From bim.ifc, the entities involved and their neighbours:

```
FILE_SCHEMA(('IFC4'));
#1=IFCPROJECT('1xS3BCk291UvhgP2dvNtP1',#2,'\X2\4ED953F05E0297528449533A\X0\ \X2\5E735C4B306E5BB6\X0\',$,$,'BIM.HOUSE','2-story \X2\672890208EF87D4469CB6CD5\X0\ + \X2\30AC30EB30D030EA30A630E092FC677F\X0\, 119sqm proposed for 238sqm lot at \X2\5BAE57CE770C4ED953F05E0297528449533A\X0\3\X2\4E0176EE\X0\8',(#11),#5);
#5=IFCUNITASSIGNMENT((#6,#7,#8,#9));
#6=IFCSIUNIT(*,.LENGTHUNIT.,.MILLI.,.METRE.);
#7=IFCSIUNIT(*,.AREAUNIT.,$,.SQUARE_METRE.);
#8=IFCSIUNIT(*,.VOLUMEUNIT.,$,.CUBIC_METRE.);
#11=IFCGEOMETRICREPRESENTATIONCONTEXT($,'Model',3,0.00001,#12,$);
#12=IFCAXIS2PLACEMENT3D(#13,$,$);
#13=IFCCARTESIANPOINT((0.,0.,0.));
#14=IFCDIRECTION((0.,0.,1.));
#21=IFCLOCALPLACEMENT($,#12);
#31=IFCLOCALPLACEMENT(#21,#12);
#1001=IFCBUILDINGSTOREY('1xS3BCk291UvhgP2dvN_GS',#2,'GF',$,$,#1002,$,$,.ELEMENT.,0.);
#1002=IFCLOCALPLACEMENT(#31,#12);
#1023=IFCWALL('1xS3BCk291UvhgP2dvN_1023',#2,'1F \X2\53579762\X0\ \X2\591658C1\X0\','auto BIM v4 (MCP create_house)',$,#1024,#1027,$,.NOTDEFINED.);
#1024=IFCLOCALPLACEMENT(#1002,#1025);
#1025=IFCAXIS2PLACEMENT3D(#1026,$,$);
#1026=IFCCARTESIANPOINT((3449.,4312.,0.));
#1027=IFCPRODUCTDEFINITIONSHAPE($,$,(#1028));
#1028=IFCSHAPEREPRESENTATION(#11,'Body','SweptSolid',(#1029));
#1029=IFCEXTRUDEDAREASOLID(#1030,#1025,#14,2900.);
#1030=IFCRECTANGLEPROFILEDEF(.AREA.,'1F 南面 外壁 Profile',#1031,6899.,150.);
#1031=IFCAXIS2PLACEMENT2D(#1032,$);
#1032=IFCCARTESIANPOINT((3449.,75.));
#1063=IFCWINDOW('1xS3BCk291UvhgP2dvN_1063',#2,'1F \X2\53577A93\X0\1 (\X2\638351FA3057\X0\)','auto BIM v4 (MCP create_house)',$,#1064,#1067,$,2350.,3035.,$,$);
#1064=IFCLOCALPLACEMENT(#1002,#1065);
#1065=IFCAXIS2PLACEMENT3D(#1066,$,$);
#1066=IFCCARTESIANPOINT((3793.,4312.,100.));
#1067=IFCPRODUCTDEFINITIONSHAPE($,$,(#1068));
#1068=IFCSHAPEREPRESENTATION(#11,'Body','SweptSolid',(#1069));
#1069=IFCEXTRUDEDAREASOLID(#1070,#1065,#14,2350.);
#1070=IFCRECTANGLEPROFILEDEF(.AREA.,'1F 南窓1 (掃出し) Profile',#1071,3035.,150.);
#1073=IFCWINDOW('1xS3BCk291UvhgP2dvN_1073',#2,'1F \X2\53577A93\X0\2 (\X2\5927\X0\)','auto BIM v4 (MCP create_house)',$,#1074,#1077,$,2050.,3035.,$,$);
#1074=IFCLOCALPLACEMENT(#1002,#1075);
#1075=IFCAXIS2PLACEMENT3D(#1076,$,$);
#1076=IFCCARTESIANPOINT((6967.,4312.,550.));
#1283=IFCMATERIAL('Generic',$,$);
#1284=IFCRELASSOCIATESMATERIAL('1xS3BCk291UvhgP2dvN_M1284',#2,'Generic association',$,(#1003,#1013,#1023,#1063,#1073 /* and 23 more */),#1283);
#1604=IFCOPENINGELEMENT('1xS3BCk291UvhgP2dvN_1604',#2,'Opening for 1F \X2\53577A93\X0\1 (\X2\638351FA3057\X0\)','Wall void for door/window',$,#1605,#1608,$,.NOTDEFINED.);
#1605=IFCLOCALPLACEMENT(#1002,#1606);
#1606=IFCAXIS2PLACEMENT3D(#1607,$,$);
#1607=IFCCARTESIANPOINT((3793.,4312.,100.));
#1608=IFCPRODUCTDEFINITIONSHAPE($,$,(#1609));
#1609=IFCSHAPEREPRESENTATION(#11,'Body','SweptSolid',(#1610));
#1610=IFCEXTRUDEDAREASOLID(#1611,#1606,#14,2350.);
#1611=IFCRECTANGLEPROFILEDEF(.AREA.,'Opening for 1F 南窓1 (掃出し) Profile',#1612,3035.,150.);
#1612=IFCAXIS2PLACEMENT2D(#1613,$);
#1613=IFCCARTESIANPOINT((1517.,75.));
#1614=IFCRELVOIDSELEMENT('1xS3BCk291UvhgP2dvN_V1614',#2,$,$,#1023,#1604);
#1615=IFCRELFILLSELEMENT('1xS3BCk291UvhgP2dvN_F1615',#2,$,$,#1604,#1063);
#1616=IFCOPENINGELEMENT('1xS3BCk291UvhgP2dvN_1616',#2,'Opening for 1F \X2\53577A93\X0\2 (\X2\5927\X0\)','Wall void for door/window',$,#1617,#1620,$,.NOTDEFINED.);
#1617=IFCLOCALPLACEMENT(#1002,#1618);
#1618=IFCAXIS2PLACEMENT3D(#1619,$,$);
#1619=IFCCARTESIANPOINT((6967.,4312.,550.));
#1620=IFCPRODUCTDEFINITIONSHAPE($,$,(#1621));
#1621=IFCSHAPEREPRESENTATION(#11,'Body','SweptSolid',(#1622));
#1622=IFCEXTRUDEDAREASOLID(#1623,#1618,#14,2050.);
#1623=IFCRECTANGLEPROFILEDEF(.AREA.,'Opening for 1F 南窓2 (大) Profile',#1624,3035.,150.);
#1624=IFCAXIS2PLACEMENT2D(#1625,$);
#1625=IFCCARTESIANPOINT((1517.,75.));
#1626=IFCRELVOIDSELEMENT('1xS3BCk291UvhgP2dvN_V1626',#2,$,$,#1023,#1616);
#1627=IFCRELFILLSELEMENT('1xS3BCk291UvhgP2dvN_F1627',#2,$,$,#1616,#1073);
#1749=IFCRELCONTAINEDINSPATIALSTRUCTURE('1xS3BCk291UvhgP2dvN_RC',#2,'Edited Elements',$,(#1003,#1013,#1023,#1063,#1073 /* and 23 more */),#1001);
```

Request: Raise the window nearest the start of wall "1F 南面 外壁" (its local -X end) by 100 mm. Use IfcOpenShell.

```python
import numpy as np
import ifcopenshell
import ifcopenshell.api.geometry
import ifcopenshell.util.placement
import ifcopenshell.util.unit

model = ifcopenshell.open("bim.ifc")
unit_scale = ifcopenshell.util.unit.calculate_unit_scale(model)

window = model.by_guid("1xS3BCk291UvhgP2dvN_1063")
opening = window.FillsVoids[0].RelatingOpeningElement
dz = 0.1 / unit_scale

shift = np.array([0.0, 0.0, dz])
# The window is not placed relative to its opening, so move both.
for product in (opening, window):
    matrix = ifcopenshell.util.placement.get_local_placement(product.ObjectPlacement)
    matrix[:3, 3] += shift
    ifcopenshell.api.geometry.edit_object_placement(model, product=product, matrix=matrix, is_si=False)

print(f"moved by {dz * unit_scale:+.3f} m")

model.write("bim_v2.ifc")
```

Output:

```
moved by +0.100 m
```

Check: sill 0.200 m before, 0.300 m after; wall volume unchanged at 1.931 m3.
